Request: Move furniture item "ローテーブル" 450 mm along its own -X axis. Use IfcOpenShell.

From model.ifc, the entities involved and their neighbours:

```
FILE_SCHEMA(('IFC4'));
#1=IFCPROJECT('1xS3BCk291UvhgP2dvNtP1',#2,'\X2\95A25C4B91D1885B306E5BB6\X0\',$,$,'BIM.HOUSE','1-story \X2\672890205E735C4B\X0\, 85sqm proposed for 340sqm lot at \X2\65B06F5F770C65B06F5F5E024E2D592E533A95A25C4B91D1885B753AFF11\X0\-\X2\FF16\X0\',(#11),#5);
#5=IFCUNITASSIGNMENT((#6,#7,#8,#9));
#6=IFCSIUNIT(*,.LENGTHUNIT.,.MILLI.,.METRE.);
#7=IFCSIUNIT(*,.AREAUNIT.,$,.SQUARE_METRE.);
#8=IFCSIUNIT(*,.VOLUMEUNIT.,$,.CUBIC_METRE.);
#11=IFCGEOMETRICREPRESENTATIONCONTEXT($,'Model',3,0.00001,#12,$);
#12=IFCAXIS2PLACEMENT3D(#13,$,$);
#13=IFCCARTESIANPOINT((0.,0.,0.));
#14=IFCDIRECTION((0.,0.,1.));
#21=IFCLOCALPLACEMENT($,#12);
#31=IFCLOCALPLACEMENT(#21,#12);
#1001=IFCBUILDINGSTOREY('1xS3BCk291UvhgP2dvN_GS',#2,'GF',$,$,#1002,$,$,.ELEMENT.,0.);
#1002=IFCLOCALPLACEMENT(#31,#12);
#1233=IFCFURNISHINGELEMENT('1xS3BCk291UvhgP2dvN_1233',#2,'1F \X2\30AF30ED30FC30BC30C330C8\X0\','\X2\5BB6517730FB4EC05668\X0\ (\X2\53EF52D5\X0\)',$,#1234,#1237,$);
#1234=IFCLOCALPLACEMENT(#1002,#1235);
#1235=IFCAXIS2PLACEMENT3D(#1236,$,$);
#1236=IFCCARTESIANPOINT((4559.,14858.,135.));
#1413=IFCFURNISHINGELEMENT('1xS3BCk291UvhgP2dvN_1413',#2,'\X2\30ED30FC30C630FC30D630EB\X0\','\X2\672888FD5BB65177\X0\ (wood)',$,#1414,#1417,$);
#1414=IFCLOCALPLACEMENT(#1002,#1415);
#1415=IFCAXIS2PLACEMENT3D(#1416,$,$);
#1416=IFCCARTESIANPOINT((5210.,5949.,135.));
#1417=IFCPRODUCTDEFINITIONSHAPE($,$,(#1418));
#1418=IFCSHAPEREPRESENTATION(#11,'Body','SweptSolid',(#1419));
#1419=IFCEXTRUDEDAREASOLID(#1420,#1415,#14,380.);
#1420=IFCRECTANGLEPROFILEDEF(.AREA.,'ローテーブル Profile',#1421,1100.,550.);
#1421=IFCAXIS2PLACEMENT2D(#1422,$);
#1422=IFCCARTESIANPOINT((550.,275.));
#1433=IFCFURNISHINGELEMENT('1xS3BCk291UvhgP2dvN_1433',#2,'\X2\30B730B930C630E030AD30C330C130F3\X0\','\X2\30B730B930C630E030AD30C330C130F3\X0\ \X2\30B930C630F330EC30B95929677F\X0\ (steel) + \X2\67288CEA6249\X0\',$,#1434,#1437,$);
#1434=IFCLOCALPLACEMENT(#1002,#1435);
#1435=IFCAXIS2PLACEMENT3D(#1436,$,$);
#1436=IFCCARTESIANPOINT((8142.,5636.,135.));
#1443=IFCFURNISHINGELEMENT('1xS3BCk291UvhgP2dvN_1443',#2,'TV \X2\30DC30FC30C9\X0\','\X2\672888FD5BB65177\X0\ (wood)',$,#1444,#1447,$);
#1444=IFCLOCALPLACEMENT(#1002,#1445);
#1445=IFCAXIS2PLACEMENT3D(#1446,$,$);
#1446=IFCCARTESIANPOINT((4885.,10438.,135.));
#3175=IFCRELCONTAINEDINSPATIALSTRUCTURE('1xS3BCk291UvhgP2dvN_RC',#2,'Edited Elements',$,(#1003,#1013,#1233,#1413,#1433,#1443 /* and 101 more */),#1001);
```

```python
import ifcopenshell
import ifcopenshell.api.geometry
import ifcopenshell.util.placement
import ifcopenshell.util.unit

model = ifcopenshell.open("model.ifc")
unit_scale = ifcopenshell.util.unit.calculate_unit_scale(model)

item = model.by_guid("1xS3BCk291UvhgP2dvN_1413")
matrix = ifcopenshell.util.placement.get_local_placement(item.ObjectPlacement)
matrix[:3, 3] -= matrix[:3, 0] * 0.45 / unit_scale
ifcopenshell.api.geometry.edit_object_placement(model, product=item, matrix=matrix, is_si=False)

print(ifcopenshell.util.placement.get_local_placement(item.ObjectPlacement).round(3) + 0.0)

model.write("model-out.ifc")
```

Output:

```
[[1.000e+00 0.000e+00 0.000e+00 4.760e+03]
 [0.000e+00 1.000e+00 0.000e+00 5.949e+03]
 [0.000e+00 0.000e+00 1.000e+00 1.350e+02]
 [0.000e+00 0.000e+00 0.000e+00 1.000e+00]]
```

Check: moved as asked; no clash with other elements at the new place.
